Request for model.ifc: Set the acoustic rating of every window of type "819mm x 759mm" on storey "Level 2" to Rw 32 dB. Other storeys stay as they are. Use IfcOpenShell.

First a look at what the model holds.

```python
import ifcopenshell
import ifcopenshell.util.element

model = ifcopenshell.open("model.ifc")
print(model.schema)
storey = next(s for s in model.by_type("IfcBuildingStorey") if s.Name == "Level 2")
windows = [e for e in ifcopenshell.util.element.get_decomposition(storey) if e.is_a("IfcWindow")]
seen = {}
for e in windows:
    element_type = ifcopenshell.util.element.get_type(e)
    key = (element_type.Name if element_type != e and element_type else None, ifcopenshell.util.element.get_pset(e, "Pset_WindowCommon", "AcousticRating"))
    seen[key] = seen.get(key, 0) + 1
for (name, value), count in sorted(seen.items(), key=str):
    print(count, "x", name, "|", value)
```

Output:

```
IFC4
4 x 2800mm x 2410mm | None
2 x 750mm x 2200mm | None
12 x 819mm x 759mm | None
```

```python
import ifcopenshell
import ifcopenshell.api.pset
import ifcopenshell.util.element

model = ifcopenshell.open("model.ifc")

storey = next(s for s in model.by_type("IfcBuildingStorey") if s.Name == "Level 2")
windows = [e for e in ifcopenshell.util.element.get_decomposition(storey) if e.is_a("IfcWindow")]

count = 0
for e in windows:
    element_type = ifcopenshell.util.element.get_type(e)
    if element_type in (None, e) or element_type.Name != "819mm x 759mm":
        continue
    # add_pset returns the element's existing set when there is one.
    pset = ifcopenshell.api.pset.add_pset(model, product=e, name="Pset_WindowCommon")
    ifcopenshell.api.pset.edit_pset(model, pset=pset, properties={"AcousticRating": "Rw 32 dB"})
    count += 1

print(count, "windows updated")

model.write("model_updated.ifc")
```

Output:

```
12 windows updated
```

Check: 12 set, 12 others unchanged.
